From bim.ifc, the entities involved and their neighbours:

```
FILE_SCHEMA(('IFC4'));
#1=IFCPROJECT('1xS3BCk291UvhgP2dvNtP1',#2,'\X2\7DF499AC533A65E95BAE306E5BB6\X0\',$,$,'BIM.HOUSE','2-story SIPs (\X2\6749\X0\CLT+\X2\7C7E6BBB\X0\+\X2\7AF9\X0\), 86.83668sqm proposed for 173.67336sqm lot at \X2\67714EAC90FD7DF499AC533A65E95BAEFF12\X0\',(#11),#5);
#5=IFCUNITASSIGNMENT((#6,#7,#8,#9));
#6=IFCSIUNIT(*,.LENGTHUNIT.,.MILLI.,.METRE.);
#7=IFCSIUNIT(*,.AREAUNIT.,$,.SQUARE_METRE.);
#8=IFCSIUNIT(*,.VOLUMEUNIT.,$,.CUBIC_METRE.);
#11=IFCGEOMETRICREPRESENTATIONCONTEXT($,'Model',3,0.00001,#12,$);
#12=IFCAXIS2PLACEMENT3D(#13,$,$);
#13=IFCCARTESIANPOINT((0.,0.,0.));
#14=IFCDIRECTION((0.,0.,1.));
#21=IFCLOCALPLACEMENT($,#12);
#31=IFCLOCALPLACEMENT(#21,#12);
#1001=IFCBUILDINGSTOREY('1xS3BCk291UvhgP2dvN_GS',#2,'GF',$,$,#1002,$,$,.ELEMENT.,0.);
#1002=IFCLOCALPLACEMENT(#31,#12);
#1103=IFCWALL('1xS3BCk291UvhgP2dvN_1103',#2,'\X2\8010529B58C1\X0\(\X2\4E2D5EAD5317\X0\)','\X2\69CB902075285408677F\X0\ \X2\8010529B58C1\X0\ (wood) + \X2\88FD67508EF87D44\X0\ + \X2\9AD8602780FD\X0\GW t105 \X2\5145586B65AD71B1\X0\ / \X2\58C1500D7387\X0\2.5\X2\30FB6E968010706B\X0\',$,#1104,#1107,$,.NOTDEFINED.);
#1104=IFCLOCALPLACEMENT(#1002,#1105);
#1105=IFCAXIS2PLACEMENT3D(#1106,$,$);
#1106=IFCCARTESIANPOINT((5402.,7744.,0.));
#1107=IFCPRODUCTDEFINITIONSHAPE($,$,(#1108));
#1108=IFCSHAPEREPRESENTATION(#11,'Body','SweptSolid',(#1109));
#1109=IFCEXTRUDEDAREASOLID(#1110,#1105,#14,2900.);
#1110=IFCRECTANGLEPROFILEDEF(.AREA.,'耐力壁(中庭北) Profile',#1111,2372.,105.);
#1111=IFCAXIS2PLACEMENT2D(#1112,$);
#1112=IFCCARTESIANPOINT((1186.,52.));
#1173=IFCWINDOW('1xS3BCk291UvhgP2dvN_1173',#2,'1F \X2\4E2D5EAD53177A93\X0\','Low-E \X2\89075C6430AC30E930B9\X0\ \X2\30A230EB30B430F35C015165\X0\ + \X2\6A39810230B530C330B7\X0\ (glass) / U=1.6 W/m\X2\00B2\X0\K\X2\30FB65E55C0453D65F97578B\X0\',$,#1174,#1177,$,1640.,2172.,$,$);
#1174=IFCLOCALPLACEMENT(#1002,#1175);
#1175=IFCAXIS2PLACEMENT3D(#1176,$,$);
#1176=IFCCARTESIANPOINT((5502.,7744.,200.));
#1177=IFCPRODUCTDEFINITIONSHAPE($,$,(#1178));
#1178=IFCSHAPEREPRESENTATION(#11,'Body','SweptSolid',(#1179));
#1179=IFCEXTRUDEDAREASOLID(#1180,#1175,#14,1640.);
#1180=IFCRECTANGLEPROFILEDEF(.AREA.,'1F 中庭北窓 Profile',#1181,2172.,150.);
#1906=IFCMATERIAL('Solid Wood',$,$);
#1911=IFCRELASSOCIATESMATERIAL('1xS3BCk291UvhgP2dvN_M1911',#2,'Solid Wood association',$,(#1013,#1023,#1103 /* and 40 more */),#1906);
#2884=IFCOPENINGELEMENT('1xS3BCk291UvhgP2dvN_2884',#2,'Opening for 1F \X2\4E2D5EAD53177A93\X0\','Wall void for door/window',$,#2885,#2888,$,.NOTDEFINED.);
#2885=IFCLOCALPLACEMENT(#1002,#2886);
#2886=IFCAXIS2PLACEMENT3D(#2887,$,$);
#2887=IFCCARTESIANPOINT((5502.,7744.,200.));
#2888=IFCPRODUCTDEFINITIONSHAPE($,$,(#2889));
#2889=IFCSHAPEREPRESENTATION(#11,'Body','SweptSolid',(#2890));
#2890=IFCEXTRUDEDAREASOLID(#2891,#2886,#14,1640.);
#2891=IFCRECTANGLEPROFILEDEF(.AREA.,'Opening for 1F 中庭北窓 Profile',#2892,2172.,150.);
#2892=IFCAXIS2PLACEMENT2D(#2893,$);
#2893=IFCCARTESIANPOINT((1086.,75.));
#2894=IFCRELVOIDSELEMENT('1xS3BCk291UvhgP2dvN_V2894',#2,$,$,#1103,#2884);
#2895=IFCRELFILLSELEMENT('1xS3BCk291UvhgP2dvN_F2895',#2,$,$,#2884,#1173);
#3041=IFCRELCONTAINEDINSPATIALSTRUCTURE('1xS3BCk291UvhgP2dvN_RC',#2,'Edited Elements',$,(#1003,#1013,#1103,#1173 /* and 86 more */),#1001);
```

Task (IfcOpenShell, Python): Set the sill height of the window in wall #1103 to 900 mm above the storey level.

```python
import numpy as np
import ifcopenshell
import ifcopenshell.api.geometry
import ifcopenshell.geom
import ifcopenshell.util.element
import ifcopenshell.util.placement
import ifcopenshell.util.shape
import ifcopenshell.util.unit

model = ifcopenshell.open("bim.ifc")
unit_scale = ifcopenshell.util.unit.calculate_unit_scale(model)

window = model.by_id(1173)
opening = window.FillsVoids[0].RelatingOpeningElement
storey = ifcopenshell.util.element.get_container(window, ifc_class="IfcBuildingStorey")
level = ifcopenshell.util.placement.get_local_placement(storey.ObjectPlacement)[2, 3]

# The opening's origin need not be at the sill, so measure its lowest point.
shape = ifcopenshell.geom.create_shape(ifcopenshell.geom.settings(), opening)
bottom = ifcopenshell.util.shape.get_shape_bottom_elevation(shape, shape.geometry) / unit_scale
dz = level + 900.0 - bottom

shift = np.array([0.0, 0.0, dz])
# The window is not placed relative to its opening, so move both.
for product in (opening, window):
    matrix = ifcopenshell.util.placement.get_local_placement(product.ObjectPlacement)
    matrix[:3, 3] += shift
    ifcopenshell.api.geometry.edit_object_placement(model, product=product, matrix=matrix, is_si=False)

print(f"moved by {dz * unit_scale:+.3f} m")

model.write("bim_updated.ifc")
```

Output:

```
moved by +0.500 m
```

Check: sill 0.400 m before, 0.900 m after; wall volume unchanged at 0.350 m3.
